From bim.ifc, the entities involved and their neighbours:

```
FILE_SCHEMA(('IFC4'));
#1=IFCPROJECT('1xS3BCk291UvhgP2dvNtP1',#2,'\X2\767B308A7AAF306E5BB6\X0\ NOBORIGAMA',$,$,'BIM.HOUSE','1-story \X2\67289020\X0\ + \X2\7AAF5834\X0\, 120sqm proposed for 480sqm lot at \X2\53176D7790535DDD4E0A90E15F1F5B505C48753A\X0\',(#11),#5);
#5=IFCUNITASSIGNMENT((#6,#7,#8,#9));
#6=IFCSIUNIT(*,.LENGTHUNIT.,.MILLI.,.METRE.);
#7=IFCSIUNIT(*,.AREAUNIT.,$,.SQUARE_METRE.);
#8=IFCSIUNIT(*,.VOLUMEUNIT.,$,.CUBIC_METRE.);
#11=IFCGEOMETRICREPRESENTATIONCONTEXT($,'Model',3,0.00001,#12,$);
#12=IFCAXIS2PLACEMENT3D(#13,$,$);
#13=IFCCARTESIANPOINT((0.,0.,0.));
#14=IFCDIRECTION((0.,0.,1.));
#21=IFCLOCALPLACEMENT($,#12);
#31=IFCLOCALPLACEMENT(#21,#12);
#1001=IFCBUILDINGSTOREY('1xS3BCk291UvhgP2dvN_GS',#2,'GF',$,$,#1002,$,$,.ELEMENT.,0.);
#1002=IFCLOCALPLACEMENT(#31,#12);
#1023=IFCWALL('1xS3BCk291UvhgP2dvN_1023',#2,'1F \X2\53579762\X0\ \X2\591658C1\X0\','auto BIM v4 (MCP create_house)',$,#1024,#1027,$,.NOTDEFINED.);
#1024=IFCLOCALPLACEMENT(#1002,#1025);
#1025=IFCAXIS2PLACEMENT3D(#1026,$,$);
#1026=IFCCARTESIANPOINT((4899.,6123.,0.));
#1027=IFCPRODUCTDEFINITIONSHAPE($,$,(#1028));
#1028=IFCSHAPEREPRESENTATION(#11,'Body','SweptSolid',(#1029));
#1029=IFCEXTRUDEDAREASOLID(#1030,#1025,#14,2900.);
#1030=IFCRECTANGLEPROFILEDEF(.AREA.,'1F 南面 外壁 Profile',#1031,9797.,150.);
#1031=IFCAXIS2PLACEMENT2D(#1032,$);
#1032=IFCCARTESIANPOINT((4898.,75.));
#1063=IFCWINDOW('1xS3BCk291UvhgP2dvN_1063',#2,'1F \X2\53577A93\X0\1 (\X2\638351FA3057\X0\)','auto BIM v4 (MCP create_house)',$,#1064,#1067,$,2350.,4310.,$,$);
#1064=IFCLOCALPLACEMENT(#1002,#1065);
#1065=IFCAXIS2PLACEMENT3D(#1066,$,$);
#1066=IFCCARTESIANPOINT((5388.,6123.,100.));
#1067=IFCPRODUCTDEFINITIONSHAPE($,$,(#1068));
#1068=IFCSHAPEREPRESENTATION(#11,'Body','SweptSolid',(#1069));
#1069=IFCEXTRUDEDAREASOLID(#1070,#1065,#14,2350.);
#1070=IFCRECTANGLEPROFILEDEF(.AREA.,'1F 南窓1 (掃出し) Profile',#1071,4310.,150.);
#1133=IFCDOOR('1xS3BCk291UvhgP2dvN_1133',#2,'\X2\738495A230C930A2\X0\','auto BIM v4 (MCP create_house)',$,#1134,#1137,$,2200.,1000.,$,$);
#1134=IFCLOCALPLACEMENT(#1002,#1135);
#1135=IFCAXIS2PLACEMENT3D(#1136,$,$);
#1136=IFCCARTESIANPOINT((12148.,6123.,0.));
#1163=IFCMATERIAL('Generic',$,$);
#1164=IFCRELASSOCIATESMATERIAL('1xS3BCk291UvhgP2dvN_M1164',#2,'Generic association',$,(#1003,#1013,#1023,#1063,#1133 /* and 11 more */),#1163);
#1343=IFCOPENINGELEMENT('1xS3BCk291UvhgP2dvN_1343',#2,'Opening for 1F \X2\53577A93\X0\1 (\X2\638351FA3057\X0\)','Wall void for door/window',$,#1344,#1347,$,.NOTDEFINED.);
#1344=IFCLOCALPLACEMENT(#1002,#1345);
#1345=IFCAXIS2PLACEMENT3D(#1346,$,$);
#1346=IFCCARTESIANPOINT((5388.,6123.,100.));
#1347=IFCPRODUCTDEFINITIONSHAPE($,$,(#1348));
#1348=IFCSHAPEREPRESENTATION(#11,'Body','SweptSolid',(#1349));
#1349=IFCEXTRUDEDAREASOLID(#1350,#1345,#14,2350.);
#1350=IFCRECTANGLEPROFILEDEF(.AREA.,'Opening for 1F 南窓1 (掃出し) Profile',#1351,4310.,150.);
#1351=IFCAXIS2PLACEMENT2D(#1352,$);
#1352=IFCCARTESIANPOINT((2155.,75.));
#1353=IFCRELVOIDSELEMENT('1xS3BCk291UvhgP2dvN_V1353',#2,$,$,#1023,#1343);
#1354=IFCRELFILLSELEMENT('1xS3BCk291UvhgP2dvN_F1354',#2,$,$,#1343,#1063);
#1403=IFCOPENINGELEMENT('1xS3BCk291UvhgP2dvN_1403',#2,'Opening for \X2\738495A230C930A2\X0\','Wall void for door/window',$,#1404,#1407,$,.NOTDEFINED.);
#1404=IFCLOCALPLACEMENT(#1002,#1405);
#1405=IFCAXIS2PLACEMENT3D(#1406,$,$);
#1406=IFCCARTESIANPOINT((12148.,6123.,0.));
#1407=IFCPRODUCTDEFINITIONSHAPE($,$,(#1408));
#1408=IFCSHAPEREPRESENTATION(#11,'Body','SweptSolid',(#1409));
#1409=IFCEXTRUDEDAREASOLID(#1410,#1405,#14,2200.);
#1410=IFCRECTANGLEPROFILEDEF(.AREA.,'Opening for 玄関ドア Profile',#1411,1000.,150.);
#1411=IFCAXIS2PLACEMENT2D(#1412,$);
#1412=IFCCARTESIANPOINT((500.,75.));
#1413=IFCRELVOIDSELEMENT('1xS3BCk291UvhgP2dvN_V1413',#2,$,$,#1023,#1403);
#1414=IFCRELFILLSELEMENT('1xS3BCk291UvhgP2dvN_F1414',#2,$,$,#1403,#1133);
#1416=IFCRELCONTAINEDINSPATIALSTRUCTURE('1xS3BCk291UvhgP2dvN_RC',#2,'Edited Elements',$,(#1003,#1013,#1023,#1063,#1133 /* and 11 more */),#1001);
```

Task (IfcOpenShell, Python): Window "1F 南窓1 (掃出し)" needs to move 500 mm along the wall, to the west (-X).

```python
import ifcopenshell
import ifcopenshell.api.geometry
import ifcopenshell.util.placement

model = ifcopenshell.open("bim.ifc")

window = model.by_guid("1xS3BCk291UvhgP2dvN_1063")
opening = window.FillsVoids[0].RelatingOpeningElement
wall = opening.VoidsElements[0].RelatingBuildingElement

wall_matrix = ifcopenshell.util.placement.get_local_placement(wall.ObjectPlacement)
shift = wall_matrix[:3, 0] * -500.0
before = ifcopenshell.util.placement.get_local_placement(window.ObjectPlacement)[:3, 3].copy()

# The window is not placed relative to its opening, so move both.
for product in (opening, window):
    matrix = ifcopenshell.util.placement.get_local_placement(product.ObjectPlacement)
    matrix[:3, 3] += shift
    ifcopenshell.api.geometry.edit_object_placement(model, product=product, matrix=matrix, is_si=False)

after = ifcopenshell.util.placement.get_local_placement(window.ObjectPlacement)[:3, 3]
print("window moved by", (after - before).round(3) + 0.0)

model.write("bim_edited.ifc")
```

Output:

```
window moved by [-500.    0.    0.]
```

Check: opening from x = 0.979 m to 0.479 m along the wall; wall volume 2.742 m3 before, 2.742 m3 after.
